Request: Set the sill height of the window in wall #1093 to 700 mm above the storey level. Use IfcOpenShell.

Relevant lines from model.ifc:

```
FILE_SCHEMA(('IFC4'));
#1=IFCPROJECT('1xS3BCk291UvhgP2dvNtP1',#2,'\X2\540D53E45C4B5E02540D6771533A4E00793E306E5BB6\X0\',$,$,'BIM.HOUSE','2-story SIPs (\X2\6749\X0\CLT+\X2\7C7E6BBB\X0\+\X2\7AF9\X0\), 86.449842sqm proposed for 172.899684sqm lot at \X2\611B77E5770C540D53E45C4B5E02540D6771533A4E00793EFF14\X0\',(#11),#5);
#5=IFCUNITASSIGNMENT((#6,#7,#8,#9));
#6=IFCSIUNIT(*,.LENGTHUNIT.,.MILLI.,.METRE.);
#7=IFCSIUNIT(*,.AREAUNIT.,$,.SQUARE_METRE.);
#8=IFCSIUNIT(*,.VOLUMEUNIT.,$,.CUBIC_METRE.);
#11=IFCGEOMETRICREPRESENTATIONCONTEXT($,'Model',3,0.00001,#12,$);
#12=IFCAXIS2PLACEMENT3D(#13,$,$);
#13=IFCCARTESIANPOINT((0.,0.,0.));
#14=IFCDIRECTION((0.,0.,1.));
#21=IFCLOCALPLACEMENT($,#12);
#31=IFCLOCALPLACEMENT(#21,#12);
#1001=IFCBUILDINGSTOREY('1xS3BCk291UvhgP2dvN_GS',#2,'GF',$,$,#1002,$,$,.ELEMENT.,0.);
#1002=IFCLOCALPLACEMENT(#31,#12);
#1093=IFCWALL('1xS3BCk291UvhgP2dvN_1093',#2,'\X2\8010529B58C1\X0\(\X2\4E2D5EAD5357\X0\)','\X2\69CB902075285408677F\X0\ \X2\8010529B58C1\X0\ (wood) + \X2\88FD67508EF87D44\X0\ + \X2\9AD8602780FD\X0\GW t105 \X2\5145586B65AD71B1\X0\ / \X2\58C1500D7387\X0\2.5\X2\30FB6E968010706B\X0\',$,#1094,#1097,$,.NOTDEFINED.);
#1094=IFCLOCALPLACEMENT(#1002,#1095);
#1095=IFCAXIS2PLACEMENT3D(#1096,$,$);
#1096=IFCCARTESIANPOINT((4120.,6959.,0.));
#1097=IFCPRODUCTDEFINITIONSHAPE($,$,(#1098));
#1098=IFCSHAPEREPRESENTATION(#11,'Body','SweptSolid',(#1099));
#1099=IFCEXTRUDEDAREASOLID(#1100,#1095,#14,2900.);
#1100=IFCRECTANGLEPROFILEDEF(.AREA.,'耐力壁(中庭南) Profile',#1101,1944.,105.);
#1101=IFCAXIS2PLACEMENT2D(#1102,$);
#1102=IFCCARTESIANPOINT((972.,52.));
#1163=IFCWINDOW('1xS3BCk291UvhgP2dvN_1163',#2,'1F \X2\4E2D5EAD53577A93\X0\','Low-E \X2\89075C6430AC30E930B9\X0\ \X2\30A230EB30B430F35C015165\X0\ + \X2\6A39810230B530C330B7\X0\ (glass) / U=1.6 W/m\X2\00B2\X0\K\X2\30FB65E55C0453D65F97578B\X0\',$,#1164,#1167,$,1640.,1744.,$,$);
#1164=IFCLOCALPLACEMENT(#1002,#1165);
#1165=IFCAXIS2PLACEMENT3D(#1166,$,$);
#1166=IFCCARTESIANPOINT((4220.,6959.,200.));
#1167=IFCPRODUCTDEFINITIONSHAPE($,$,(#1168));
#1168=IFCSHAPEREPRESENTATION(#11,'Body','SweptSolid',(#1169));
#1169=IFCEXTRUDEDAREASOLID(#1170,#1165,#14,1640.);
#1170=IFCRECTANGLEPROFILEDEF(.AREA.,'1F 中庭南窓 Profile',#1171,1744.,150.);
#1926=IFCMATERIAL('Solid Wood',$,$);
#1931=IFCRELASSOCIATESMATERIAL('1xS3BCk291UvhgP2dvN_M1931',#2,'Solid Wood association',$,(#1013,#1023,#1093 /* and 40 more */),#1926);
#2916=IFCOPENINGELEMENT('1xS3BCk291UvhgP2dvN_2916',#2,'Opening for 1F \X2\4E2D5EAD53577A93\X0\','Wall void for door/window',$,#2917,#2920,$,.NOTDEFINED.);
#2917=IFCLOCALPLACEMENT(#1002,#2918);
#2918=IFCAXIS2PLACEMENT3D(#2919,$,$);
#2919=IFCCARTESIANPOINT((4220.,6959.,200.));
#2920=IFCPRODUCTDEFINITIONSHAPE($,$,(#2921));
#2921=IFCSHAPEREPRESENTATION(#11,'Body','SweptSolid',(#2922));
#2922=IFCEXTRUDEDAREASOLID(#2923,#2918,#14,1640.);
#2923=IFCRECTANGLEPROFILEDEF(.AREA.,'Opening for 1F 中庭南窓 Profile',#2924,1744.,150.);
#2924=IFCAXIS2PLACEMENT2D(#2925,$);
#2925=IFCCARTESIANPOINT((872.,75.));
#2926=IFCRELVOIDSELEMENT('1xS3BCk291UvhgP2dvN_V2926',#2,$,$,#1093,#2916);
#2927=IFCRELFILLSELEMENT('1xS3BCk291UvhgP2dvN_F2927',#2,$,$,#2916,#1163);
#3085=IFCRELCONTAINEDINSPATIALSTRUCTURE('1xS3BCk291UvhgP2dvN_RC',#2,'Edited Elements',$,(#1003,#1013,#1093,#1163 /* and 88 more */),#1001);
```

```python
import numpy as np
import ifcopenshell
import ifcopenshell.api.geometry
import ifcopenshell.geom
import ifcopenshell.util.element
import ifcopenshell.util.placement
import ifcopenshell.util.shape
import ifcopenshell.util.unit

model = ifcopenshell.open("model.ifc")
unit_scale = ifcopenshell.util.unit.calculate_unit_scale(model)

window = model.by_guid("1xS3BCk291UvhgP2dvN_1163")
opening = window.FillsVoids[0].RelatingOpeningElement
storey = ifcopenshell.util.element.get_container(window, ifc_class="IfcBuildingStorey")
level = ifcopenshell.util.placement.get_local_placement(storey.ObjectPlacement)[2, 3]

# The opening's origin need not be at the sill, so measure its lowest point.
shape = ifcopenshell.geom.create_shape(ifcopenshell.geom.settings(), opening)
bottom = ifcopenshell.util.shape.get_shape_bottom_elevation(shape, shape.geometry) / unit_scale
dz = level + 0.7 / unit_scale - bottom

shift = np.array([0.0, 0.0, dz])
# The window is not placed relative to its opening, so move both.
for product in (opening, window):
    matrix = ifcopenshell.util.placement.get_local_placement(product.ObjectPlacement)
    matrix[:3, 3] += shift
    ifcopenshell.api.geometry.edit_object_placement(model, product=product, matrix=matrix, is_si=False)

print(f"moved by {dz * unit_scale:+.3f} m")

model.write("model_edited.ifc")
```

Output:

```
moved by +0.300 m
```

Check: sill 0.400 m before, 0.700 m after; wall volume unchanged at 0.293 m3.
